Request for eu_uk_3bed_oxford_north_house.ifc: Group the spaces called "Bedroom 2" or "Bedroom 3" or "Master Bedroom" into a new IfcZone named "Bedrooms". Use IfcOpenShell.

First a look at what the model holds.

```python
import ifcopenshell

model = ifcopenshell.open("eu_uk_3bed_oxford_north_house.ifc")
print(model.schema)
seen = {}
for space in model.by_type("IfcSpace"):
    seen[space.LongName] = seen.get(space.LongName, 0) + 1
for name, count in sorted(seen.items(), key=str):
    print(count, "x", name)
print("zones:", [z.Name for z in model.by_type("IfcZone")][:20])
```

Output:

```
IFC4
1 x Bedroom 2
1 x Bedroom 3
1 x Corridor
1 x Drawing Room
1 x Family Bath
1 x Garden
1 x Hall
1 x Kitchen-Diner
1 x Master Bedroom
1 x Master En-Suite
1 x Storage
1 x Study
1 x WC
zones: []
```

```python
import ifcopenshell
import ifcopenshell.api.group
import ifcopenshell.api.root

model = ifcopenshell.open("eu_uk_3bed_oxford_north_house.ifc")

names = {"Bedroom 2", "Bedroom 3", "Master Bedroom"}
spaces = [s for s in model.by_type("IfcSpace") if s.LongName in names]

zone = ifcopenshell.api.root.create_entity(model, ifc_class="IfcZone", name="Bedrooms")
ifcopenshell.api.group.assign_group(model, products=spaces, group=zone)
print(len(spaces), "spaces in", zone.Name)

model.write("eu_uk_3bed_oxford_north_house_v2.ifc")
```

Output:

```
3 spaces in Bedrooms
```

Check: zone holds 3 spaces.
